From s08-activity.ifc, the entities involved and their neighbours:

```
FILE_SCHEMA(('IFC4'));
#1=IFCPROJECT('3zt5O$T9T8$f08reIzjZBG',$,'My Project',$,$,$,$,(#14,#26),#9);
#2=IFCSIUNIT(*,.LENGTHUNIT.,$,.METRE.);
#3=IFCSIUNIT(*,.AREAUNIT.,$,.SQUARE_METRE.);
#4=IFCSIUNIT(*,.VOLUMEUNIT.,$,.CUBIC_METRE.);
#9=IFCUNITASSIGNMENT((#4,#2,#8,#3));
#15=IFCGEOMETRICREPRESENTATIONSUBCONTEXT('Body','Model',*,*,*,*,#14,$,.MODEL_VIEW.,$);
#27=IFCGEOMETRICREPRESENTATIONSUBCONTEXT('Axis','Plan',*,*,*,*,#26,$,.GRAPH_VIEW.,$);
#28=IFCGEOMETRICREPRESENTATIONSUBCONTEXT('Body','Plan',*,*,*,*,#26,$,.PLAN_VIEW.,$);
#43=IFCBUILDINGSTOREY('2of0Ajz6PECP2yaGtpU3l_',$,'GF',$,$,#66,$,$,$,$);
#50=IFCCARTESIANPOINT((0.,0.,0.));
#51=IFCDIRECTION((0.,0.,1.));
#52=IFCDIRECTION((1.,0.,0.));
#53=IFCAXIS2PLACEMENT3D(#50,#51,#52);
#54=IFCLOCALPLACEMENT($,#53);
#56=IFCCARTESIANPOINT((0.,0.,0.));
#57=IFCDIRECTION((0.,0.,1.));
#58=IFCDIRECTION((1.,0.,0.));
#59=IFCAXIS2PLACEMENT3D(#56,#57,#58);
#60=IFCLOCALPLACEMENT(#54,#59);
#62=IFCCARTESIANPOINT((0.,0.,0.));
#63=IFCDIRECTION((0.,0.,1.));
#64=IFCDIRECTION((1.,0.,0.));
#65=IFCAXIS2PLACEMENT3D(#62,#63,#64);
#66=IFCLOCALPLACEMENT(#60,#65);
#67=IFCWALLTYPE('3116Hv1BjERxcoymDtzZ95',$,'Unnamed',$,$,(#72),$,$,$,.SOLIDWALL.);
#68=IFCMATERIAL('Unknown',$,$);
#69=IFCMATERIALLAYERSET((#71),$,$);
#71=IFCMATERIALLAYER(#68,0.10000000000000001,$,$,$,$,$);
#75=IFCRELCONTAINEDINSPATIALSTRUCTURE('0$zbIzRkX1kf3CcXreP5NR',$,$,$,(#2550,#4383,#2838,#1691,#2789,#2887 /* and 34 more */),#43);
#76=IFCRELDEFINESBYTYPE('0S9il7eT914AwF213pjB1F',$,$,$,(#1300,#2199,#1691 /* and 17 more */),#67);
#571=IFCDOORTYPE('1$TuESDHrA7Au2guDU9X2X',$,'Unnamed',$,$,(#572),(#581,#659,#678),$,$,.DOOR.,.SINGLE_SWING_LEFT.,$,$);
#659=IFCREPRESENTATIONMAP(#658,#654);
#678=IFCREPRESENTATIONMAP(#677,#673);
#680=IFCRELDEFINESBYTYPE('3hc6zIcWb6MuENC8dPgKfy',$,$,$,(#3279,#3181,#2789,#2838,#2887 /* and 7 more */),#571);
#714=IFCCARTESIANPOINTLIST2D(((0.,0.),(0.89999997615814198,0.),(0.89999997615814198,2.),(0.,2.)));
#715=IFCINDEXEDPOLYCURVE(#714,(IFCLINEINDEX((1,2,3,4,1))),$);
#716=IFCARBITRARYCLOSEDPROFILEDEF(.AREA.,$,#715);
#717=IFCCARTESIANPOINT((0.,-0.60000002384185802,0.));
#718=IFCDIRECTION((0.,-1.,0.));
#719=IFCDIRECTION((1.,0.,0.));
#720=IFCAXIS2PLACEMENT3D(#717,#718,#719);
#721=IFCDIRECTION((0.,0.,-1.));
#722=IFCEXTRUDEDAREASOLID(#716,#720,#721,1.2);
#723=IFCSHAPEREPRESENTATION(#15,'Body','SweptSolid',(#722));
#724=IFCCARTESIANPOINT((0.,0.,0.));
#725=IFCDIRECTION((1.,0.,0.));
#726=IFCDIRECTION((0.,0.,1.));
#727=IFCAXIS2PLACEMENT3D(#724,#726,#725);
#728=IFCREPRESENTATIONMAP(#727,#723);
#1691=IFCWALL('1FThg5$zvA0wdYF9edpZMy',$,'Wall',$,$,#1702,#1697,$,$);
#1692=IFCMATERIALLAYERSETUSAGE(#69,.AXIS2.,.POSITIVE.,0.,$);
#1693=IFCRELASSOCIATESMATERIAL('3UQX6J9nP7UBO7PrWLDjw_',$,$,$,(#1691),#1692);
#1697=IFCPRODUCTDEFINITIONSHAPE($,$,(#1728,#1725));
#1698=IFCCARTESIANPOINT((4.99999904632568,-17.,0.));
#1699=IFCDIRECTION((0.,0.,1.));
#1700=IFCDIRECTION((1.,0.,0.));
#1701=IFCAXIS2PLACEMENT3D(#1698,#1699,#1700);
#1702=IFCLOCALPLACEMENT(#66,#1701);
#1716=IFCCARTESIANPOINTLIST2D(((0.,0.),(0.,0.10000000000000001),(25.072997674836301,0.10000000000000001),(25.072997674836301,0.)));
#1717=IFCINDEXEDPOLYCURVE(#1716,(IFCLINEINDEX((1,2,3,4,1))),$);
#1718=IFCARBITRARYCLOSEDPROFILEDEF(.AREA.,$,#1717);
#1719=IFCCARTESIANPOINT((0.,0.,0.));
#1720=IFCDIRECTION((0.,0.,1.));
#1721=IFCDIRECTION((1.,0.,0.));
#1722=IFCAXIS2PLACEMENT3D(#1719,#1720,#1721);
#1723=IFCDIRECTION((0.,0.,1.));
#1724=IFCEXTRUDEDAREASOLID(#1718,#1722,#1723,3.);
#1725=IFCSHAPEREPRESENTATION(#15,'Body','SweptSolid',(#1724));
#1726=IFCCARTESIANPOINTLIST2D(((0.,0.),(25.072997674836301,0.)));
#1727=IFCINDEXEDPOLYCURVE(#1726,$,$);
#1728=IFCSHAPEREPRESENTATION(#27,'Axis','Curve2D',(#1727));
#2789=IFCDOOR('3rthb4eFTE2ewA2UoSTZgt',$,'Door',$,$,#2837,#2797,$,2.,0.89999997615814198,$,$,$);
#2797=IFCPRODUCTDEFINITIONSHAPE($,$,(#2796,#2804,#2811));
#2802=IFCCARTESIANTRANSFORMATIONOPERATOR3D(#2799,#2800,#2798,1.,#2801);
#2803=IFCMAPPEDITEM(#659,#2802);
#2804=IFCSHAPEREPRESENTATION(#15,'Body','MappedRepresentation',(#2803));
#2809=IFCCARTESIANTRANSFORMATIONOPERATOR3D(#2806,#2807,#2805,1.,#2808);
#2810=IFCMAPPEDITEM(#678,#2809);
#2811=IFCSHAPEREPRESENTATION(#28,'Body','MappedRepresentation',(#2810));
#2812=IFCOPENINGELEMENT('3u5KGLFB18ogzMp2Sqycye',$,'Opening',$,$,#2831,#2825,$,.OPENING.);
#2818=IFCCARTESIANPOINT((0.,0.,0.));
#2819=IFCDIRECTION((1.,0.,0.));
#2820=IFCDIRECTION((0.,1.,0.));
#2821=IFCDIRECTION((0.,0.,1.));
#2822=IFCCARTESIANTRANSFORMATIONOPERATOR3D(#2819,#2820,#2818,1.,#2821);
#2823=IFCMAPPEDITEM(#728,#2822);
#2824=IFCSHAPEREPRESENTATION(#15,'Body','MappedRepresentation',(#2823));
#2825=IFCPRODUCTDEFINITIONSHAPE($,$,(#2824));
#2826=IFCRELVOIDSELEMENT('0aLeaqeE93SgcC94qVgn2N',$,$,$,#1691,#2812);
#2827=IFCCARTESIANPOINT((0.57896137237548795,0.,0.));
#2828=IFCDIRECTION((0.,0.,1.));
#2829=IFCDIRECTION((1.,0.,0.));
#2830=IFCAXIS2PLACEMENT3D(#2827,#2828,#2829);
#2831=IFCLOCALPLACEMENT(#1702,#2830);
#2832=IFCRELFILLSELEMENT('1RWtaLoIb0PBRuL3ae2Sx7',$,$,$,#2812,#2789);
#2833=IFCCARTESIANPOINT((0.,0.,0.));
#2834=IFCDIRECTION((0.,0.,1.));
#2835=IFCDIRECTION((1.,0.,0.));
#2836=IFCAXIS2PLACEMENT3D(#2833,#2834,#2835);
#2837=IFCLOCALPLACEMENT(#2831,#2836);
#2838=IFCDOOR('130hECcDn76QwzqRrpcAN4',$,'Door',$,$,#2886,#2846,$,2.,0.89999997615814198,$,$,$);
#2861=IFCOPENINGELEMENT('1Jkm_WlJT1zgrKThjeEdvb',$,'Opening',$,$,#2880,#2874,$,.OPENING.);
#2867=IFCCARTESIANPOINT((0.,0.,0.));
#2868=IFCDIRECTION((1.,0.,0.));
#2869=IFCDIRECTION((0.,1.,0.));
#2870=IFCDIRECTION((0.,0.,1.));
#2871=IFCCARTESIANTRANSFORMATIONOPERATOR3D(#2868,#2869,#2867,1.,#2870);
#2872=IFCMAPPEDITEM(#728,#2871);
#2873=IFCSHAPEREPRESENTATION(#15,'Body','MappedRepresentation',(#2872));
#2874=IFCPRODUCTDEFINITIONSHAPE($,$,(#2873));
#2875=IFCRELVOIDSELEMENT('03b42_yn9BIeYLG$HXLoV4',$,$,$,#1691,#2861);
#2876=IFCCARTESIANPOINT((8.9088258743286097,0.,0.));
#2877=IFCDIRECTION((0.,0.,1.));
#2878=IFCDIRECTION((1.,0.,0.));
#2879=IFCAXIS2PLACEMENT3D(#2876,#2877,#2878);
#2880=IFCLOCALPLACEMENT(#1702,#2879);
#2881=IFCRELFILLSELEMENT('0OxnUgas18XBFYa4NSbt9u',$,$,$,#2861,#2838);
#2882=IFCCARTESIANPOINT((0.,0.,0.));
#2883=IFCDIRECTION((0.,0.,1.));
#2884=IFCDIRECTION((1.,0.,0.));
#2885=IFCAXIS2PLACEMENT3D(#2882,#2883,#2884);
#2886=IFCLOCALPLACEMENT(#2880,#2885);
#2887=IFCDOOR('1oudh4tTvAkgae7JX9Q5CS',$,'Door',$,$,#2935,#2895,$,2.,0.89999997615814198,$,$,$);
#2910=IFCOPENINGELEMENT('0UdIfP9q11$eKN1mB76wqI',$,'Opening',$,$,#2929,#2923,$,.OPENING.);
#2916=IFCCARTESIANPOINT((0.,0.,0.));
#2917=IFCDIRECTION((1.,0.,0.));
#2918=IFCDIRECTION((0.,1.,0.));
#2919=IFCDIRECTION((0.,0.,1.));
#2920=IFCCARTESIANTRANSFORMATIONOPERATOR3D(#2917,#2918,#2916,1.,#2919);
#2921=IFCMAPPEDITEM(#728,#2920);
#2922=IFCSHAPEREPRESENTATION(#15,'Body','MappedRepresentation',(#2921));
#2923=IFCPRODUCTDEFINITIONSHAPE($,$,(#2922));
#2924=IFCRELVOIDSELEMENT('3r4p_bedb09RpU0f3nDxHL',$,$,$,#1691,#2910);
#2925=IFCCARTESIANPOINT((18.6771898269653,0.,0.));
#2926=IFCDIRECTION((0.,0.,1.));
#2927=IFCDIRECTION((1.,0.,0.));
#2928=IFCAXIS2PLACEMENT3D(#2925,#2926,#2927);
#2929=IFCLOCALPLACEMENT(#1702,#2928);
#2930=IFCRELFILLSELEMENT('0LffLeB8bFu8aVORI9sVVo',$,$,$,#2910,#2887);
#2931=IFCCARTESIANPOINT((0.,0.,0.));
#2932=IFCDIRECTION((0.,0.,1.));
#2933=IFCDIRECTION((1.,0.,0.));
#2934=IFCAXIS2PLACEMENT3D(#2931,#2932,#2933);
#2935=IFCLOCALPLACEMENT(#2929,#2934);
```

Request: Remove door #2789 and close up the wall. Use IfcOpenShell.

```python
import ifcopenshell
import ifcopenshell.api.feature
import ifcopenshell.api.root
import ifcopenshell.geom
import ifcopenshell.util.shape

model = ifcopenshell.open("s08-activity.ifc")
settings = ifcopenshell.geom.settings()


def volume(element):
    """Net volume in cubic metres, openings subtracted."""
    shape = ifcopenshell.geom.create_shape(settings, element)
    return ifcopenshell.util.shape.get_volume(shape.geometry)


door = model.by_guid("3rthb4eFTE2ewA2UoSTZgt")
opening = door.FillsVoids[0].RelatingOpeningElement
wall = opening.VoidsElements[0].RelatingBuildingElement
before = volume(wall)

ifcopenshell.api.root.remove_product(model, product=door)
ifcopenshell.api.feature.remove_feature(model, feature=opening)

after = volume(wall)

print(f"wall volume {before:.3f} -> {after:.3f} m3")

model.write("s08-activity-out.ifc")
```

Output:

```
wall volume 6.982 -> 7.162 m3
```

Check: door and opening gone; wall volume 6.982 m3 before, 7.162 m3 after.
